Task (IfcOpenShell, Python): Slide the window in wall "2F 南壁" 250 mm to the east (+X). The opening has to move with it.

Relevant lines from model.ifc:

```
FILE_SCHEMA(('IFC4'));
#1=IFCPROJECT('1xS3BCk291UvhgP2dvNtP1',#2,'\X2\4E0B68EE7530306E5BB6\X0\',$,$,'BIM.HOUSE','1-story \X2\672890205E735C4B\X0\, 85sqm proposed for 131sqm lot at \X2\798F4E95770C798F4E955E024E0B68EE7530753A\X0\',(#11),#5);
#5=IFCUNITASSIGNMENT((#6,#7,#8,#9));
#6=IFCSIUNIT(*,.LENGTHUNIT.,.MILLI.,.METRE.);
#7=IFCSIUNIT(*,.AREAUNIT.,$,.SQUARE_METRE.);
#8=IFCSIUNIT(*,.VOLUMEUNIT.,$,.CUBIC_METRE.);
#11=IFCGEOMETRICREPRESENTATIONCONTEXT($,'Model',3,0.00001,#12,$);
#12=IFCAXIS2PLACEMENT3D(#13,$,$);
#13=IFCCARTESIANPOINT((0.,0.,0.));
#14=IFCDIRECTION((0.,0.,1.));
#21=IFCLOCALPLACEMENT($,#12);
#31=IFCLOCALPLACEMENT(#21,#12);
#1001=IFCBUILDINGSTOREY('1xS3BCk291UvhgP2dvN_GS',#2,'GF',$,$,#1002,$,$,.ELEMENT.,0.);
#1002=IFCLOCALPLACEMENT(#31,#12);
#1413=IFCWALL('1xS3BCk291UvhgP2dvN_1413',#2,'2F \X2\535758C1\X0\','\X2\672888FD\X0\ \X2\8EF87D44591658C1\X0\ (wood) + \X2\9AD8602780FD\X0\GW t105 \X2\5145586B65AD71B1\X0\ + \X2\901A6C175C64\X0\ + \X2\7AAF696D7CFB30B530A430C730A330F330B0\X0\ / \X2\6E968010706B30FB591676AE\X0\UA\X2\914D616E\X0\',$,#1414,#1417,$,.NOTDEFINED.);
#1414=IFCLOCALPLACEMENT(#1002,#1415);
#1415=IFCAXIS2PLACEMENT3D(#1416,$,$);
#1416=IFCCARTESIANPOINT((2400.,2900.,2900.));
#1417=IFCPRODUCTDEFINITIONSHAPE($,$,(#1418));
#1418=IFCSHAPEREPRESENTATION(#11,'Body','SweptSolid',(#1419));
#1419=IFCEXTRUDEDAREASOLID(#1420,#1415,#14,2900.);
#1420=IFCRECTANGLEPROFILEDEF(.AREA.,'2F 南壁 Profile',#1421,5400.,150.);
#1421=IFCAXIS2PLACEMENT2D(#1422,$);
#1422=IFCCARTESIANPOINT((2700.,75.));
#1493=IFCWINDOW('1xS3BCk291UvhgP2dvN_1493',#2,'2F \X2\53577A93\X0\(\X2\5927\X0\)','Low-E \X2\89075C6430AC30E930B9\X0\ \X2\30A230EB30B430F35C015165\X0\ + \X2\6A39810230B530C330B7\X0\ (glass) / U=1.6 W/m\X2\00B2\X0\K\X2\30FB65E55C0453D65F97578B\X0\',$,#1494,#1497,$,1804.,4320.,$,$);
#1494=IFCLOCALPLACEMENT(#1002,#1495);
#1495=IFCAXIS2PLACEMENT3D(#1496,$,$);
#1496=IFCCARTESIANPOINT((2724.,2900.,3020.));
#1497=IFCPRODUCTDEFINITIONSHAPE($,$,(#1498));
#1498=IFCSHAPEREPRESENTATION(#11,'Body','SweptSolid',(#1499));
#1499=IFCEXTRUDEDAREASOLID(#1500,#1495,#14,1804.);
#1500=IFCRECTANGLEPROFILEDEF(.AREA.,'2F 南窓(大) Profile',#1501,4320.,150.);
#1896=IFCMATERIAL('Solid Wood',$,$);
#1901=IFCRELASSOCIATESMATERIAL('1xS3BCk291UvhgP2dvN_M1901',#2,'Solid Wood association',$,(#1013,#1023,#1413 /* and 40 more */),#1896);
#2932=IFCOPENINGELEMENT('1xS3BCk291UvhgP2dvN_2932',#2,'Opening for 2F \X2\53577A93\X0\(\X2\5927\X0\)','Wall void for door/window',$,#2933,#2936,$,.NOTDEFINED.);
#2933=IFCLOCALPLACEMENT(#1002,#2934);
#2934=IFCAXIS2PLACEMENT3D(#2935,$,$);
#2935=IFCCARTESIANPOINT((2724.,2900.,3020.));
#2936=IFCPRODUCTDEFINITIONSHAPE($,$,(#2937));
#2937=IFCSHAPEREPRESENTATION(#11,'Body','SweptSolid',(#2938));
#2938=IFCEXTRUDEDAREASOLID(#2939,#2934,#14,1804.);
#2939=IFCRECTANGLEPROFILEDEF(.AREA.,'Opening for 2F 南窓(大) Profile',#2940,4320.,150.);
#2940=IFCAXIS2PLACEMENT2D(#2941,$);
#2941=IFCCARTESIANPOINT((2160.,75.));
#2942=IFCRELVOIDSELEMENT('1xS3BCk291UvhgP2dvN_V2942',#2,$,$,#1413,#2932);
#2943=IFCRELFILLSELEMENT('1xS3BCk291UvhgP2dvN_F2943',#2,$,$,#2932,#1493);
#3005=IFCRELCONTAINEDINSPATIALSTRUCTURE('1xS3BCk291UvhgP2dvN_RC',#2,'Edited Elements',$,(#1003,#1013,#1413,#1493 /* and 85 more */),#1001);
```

```python
import ifcopenshell
import ifcopenshell.api.geometry
import ifcopenshell.util.placement

model = ifcopenshell.open("model.ifc")

window = model.by_guid("1xS3BCk291UvhgP2dvN_1493")
opening = window.FillsVoids[0].RelatingOpeningElement
wall = opening.VoidsElements[0].RelatingBuildingElement

wall_matrix = ifcopenshell.util.placement.get_local_placement(wall.ObjectPlacement)
shift = wall_matrix[:3, 0] * 250.0
before = ifcopenshell.util.placement.get_local_placement(window.ObjectPlacement)[:3, 3].copy()

# The window is not placed relative to its opening, so move both.
for product in (opening, window):
    matrix = ifcopenshell.util.placement.get_local_placement(product.ObjectPlacement)
    matrix[:3, 3] += shift
    ifcopenshell.api.geometry.edit_object_placement(model, product=product, matrix=matrix, is_si=False)

after = ifcopenshell.util.placement.get_local_placement(window.ObjectPlacement)[:3, 3]
print("window moved by", (after - before).round(3) + 0.0)

model.write("model_edited.ifc")
```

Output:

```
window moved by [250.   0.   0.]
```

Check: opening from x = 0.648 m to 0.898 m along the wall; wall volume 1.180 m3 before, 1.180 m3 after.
